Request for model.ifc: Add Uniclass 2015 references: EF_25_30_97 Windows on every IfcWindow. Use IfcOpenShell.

First a look at what the model holds.

```python
import ifcopenshell

model = ifcopenshell.open("model.ifc")
print(model.schema)
print("classifications:", [c.Name for c in model.by_type("IfcClassification")])
for ifc_class in ("IfcDoor", "IfcRoof", "IfcStair", "IfcWall", "IfcWindow"):
    print(ifc_class, len(model.by_type(ifc_class)))
```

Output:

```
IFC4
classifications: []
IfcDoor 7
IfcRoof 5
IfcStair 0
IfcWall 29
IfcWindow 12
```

```python
import ifcopenshell
import ifcopenshell.api.classification

model = ifcopenshell.open("model.ifc")

system = ifcopenshell.api.classification.add_classification(model, classification="Uniclass 2015")

codes = {
    "IfcWindow": ("EF_25_30_97", "Windows"),
}
for ifc_class, (code, name) in codes.items():
    products = model.by_type(ifc_class)
    ifcopenshell.api.classification.add_reference(
        model, products=products, classification=system, identification=code, name=name
    )
    print(code, len(products))

model.write("model_updated.ifc")
```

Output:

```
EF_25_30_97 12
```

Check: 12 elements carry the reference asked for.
